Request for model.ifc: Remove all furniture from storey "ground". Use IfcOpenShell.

First a look at what the model holds.

```python
import ifcopenshell
import ifcopenshell.util.element

model = ifcopenshell.open("model.ifc")
print(model.schema)
storey = next(s for s in model.by_type("IfcBuildingStorey") if s.Name == "ground")
furniture = [e for e in ifcopenshell.util.element.get_decomposition(storey) if e.is_a("IfcFurnishingElement")]
seen = {}
for e in furniture:
    element_type = ifcopenshell.util.element.get_type(e)
    name = element_type.Name if element_type not in (None, e) else None
    seen[name] = seen.get(name, 0) + 1
for name, count in sorted(seen.items(), key=str):
    print(count, "x", name)
```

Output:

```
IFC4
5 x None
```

```python
import ifcopenshell
import ifcopenshell.api.root
import ifcopenshell.util.element

model = ifcopenshell.open("model.ifc")

storey = next(s for s in model.by_type("IfcBuildingStorey") if s.Name == "ground")
furniture = [e for e in ifcopenshell.util.element.get_decomposition(storey) if e.is_a("IfcFurnishingElement")]

for e in furniture:
    ifcopenshell.api.root.remove_product(model, product=e)
print(len(furniture), "removed")

model.write("model_v2.ifc")
```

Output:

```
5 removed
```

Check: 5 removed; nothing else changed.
